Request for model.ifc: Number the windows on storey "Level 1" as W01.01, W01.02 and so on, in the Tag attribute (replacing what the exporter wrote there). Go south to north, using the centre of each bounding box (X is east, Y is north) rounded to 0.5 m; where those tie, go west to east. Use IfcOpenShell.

First a look at what the model holds.

```python
import ifcopenshell
import ifcopenshell.util.element
import ifcopenshell.util.placement

model = ifcopenshell.open("model.ifc")
print(model.schema)
storey = next(s for s in model.by_type("IfcBuildingStorey") if s.Name == "Level 1")
windows = [e for e in ifcopenshell.util.element.get_decomposition(storey) if e.is_a("IfcWindow")]
for e in sorted(windows, key=lambda e: e.id()):
    origin = ifcopenshell.util.placement.get_local_placement(e.ObjectPlacement)[:3, 3]
    print(e.id(), e.Tag, e.Name, origin.round(2) + 0.0, sep=" | ")
```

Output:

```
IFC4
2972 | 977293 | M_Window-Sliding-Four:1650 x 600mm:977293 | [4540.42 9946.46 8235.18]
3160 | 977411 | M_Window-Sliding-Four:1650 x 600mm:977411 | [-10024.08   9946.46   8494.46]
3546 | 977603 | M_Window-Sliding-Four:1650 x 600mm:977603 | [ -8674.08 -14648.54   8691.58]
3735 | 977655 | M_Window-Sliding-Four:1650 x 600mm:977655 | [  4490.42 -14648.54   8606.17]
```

```python
import ifcopenshell
import ifcopenshell.geom
import ifcopenshell.util.element
import ifcopenshell.util.shape

model = ifcopenshell.open("model.ifc")
settings = ifcopenshell.geom.settings()
settings.set("use-world-coords", True)


def centre(element):
    shape = ifcopenshell.geom.create_shape(settings, element)
    return ifcopenshell.util.shape.get_bbox_centroid(shape.geometry)


storey = next(s for s in model.by_type("IfcBuildingStorey") if s.Name == "Level 1")
windows = [e for e in ifcopenshell.util.element.get_decomposition(storey) if e.is_a("IfcWindow")]

# Insertion points can sit at a corner or the storey origin, so sort by the geometry (in metres).
centres = {e: centre(e) for e in windows}
windows.sort(key=lambda e: (round(centres[e][1] / 0.5), centres[e][0]))

for i, e in enumerate(windows, start=1):
    number = f"W01.{i:02d}"
    e.Tag = number
    print(e.id(), number)

model.write("model-out.ifc")
```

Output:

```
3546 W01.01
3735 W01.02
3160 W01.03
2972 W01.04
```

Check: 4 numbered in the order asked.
